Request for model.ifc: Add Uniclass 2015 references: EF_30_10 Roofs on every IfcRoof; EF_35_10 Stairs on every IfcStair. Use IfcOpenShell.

First a look at what the model holds.

```python
import ifcopenshell

model = ifcopenshell.open("model.ifc")
print(model.schema)
print("classifications:", [c.Name for c in model.by_type("IfcClassification")])
for ifc_class in ("IfcDoor", "IfcRoof", "IfcStair", "IfcWall", "IfcWindow"):
    print(ifc_class, len(model.by_type(ifc_class)))
```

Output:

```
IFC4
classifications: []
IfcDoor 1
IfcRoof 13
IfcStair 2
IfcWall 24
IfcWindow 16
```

```python
import ifcopenshell
import ifcopenshell.api.classification

model = ifcopenshell.open("model.ifc")

system = ifcopenshell.api.classification.add_classification(model, classification="Uniclass 2015")

codes = {
    "IfcRoof": ("EF_30_10", "Roofs"),
    "IfcStair": ("EF_35_10", "Stairs"),
}
for ifc_class, (code, name) in codes.items():
    products = model.by_type(ifc_class)
    ifcopenshell.api.classification.add_reference(
        model, products=products, classification=system, identification=code, name=name
    )
    print(code, len(products))

model.write("model_v2.ifc")
```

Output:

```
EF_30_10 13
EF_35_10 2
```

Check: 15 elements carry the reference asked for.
